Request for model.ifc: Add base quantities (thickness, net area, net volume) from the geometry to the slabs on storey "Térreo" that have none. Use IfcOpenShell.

First a look at what the model holds.

```python
import ifcopenshell
import ifcopenshell.util.element
import ifcopenshell.util.unit

model = ifcopenshell.open("model.ifc")
print(model.schema)
for unit_type in ("LENGTHUNIT", "AREAUNIT", "VOLUMEUNIT"):
    print(unit_type, ifcopenshell.util.unit.calculate_unit_scale(model, unit_type))
storey = next(s for s in model.by_type("IfcBuildingStorey") if s.Name == "Térreo")
slabs = [e for e in ifcopenshell.util.element.get_decomposition(storey) if e.is_a("IfcSlab")]
for e in sorted(slabs, key=lambda e: e.id()):
    print(e.id(), e.is_a(), e.Name, list(ifcopenshell.util.element.get_psets(e, qtos_only=True)), sep=" | ")
```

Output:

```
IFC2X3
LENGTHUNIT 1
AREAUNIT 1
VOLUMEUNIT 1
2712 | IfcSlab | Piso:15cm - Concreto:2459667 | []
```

```python
import ifcopenshell
import ifcopenshell.api.pset
import ifcopenshell.geom
import ifcopenshell.util.element
import ifcopenshell.util.shape
import ifcopenshell.util.unit

model = ifcopenshell.open("model.ifc")
unit_scale = ifcopenshell.util.unit.calculate_unit_scale(model)
area_scale = ifcopenshell.util.unit.calculate_unit_scale(model, "AREAUNIT")
volume_scale = ifcopenshell.util.unit.calculate_unit_scale(model, "VOLUMEUNIT")
settings = ifcopenshell.geom.settings()

storey = next(s for s in model.by_type("IfcBuildingStorey") if s.Name == "Térreo")
slabs = [e for e in ifcopenshell.util.element.get_decomposition(storey) if e.is_a("IfcSlab")]

for e in sorted(slabs, key=lambda e: e.id()):
    if ifcopenshell.util.element.get_psets(e, qtos_only=True, should_inherit=False):
        continue
    # Geometry comes back in metres, in the element's own axes.
    shape = ifcopenshell.geom.create_shape(settings, e)
    values = {
        "Width": ifcopenshell.util.shape.get_z(shape.geometry) / unit_scale,
        "NetArea": ifcopenshell.util.shape.get_footprint_area(shape.geometry) / area_scale,
        "NetVolume": ifcopenshell.util.shape.get_volume(shape.geometry) / volume_scale,
    }
    qto = ifcopenshell.api.pset.add_qto(model, product=e, name="BaseQuantities")
    ifcopenshell.api.pset.edit_qto(model, qto=qto, properties=values)
    print(e.id(), {k: round(v, 3) for k, v in values.items()})

model.write("model-out.ifc")
```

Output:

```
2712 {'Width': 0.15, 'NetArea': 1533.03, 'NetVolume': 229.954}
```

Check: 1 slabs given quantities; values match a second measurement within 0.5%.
